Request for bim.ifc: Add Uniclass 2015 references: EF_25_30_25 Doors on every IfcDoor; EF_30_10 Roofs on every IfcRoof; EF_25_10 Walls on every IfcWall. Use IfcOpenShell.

First a look at what the model holds.

```python
import ifcopenshell

model = ifcopenshell.open("bim.ifc")
print(model.schema)
print("classifications:", [c.Name for c in model.by_type("IfcClassification")])
for ifc_class in ("IfcDoor", "IfcRoof", "IfcStair", "IfcWall", "IfcWindow"):
    print(ifc_class, len(model.by_type(ifc_class)))
```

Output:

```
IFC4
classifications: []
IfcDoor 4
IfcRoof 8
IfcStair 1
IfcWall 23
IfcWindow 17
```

```python
import ifcopenshell
import ifcopenshell.api.classification

model = ifcopenshell.open("bim.ifc")

system = ifcopenshell.api.classification.add_classification(model, classification="Uniclass 2015")

codes = {
    "IfcDoor": ("EF_25_30_25", "Doors"),
    "IfcRoof": ("EF_30_10", "Roofs"),
    "IfcWall": ("EF_25_10", "Walls"),
}
for ifc_class, (code, name) in codes.items():
    products = model.by_type(ifc_class)
    ifcopenshell.api.classification.add_reference(
        model, products=products, classification=system, identification=code, name=name
    )
    print(code, len(products))

model.write("bim_updated.ifc")
```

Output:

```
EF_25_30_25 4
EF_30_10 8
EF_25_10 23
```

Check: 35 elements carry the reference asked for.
